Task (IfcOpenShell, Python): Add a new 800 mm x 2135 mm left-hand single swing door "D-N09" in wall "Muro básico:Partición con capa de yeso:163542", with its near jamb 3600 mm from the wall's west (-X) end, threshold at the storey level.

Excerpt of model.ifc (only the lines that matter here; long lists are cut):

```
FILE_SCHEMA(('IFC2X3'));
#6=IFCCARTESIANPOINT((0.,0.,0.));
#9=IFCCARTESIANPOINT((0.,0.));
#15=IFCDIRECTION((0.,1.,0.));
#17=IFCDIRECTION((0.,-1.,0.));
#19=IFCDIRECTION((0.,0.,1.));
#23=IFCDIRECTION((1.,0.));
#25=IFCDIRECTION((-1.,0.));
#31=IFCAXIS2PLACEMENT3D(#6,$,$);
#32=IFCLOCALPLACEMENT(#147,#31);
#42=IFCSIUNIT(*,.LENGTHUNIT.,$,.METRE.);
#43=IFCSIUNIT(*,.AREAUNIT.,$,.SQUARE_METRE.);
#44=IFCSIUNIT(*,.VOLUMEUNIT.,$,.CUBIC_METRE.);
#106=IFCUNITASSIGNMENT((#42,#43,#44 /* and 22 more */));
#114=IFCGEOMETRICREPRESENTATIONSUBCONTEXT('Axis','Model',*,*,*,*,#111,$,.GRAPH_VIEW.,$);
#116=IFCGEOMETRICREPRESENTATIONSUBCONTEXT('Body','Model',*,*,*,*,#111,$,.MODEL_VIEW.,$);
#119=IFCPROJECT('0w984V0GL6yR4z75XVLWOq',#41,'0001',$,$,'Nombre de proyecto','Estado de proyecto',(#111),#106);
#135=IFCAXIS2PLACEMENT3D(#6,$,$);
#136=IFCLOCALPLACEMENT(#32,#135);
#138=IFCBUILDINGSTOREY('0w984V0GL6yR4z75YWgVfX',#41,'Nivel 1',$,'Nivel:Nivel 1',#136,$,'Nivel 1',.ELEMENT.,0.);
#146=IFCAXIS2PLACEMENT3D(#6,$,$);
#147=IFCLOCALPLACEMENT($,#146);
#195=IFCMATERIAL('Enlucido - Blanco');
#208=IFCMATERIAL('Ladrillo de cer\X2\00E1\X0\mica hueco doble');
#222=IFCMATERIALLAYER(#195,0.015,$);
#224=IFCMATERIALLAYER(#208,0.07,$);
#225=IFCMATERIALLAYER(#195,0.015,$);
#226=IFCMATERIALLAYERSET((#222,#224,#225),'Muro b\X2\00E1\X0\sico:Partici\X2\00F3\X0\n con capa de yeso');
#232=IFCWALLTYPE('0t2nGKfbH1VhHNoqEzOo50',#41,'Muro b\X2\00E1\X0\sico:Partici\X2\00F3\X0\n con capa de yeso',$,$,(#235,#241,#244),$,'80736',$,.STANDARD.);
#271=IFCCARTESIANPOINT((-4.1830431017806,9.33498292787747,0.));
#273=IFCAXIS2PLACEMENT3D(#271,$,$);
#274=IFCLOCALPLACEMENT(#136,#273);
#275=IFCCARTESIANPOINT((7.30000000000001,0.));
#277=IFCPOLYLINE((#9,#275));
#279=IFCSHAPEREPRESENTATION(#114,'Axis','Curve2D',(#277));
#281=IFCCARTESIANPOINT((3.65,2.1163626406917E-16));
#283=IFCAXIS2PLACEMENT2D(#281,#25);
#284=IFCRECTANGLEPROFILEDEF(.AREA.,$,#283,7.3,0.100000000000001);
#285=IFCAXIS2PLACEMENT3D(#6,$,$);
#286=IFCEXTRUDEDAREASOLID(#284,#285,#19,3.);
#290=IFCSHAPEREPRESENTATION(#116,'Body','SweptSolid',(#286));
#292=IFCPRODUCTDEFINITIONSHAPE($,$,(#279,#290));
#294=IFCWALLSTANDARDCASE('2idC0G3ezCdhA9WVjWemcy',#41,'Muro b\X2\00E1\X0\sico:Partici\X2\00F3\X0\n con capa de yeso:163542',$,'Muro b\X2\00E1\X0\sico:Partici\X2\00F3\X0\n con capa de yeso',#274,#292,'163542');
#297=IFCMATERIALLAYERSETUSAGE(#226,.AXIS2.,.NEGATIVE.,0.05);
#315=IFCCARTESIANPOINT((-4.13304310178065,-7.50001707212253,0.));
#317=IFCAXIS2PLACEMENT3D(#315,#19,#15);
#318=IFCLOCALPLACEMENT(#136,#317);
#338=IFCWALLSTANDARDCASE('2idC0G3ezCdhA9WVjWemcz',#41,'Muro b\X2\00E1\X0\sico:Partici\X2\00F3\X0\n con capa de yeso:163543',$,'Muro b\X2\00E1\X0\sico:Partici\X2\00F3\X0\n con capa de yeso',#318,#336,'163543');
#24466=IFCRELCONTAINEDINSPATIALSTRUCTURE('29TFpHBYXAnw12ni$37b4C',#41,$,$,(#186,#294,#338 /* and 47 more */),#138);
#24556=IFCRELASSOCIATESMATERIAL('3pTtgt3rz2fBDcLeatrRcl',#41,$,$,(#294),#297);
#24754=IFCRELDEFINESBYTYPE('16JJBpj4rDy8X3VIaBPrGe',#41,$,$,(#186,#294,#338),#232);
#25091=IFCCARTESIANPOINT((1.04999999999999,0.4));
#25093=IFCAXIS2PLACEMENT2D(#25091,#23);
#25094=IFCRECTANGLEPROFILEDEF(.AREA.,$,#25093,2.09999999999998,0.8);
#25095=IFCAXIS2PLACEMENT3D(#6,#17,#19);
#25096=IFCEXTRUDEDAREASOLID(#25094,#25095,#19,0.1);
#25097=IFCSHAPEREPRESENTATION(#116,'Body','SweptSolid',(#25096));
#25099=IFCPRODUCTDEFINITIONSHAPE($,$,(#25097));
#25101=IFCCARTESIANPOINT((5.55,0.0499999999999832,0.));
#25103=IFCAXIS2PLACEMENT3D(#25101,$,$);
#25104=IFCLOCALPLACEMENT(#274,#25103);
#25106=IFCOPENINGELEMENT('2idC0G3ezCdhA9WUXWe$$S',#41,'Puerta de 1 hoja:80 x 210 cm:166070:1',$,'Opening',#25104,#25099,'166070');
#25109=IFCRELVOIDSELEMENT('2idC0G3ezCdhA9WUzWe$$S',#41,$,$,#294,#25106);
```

```python
import numpy as np
import ifcopenshell
import ifcopenshell.api.feature
import ifcopenshell.api.geometry
import ifcopenshell.api.root
import ifcopenshell.api.spatial
import ifcopenshell.api.type
import ifcopenshell.geom
import ifcopenshell.util.element
import ifcopenshell.util.placement
import ifcopenshell.util.representation
import ifcopenshell.util.shape
import ifcopenshell.util.unit

model = ifcopenshell.open("model.ifc")
unit_scale = ifcopenshell.util.unit.calculate_unit_scale(model)
settings = ifcopenshell.geom.settings()


def volume(element):
    """Net volume in cubic metres, openings subtracted."""
    shape = ifcopenshell.geom.create_shape(settings, element)
    return ifcopenshell.util.shape.get_volume(shape.geometry)


wall = model.by_guid("2idC0G3ezCdhA9WVjWemcy")
storey = ifcopenshell.util.element.get_container(wall, ifc_class="IfcBuildingStorey")
context = ifcopenshell.util.representation.get_context(model, "Model", "Body", "MODEL_VIEW")
before = volume(wall)

width, height, from_end, sill = 0.8, 2.135, 3.6, 0.0  # metres

# The wall runs along its own X axis, and the end named is its -X end.
wall_shape = ifcopenshell.geom.create_shape(settings, wall)
x, y, z = ifcopenshell.util.shape.get_vertices(wall_shape.geometry).T
start = x.min() + from_end
face, thickness = float(y.min()), float(y.max() - y.min())
wall_matrix = ifcopenshell.util.placement.get_local_placement(wall.ObjectPlacement)
level = ifcopenshell.util.placement.get_local_placement(storey.ObjectPlacement)[2, 3]


def in_wall(x, y):
    """Placement at x, y metres in the wall's axes, at sill height."""
    matrix = wall_matrix.copy()
    matrix[:, 3] = wall_matrix @ np.array([x / unit_scale, y / unit_scale, 0.0, 1.0])
    matrix[2, 3] = level + sill / unit_scale
    return matrix


# Opening: a box that overshoots both wall faces by 50 mm.
opening = ifcopenshell.api.root.create_entity(model, ifc_class="IfcOpeningElement")
box = ifcopenshell.api.geometry.add_wall_representation(
    model, context=context, length=width, height=height, thickness=thickness + 0.1
)
ifcopenshell.api.geometry.assign_representation(model, product=opening, representation=box)
ifcopenshell.api.geometry.edit_object_placement(model, product=opening, matrix=in_wall(start, face - 0.05), is_si=False)
ifcopenshell.api.feature.add_feature(model, feature=opening, element=wall)

door = ifcopenshell.api.root.create_entity(model, ifc_class="IfcDoor", name="D-N09")
door.OverallWidth, door.OverallHeight = width / unit_scale, height / unit_scale
body = ifcopenshell.api.geometry.add_door_representation(
    model,
    context=context,
    overall_width=door.OverallWidth,
    overall_height=door.OverallHeight,
    operation_type="SINGLE_SWING_LEFT",
    lining_properties={"LiningDepth": thickness / unit_scale, "ThresholdDepth": thickness / unit_scale},
)
ifcopenshell.api.geometry.assign_representation(model, product=door, representation=body)
ifcopenshell.api.spatial.assign_container(model, products=[door], relating_structure=storey)
fills = ifcopenshell.api.feature.add_filling(model, opening=opening, element=door)
fills.OwnerHistory = door.OwnerHistory  # required in IFC2X3

# IFC2X3 keeps the operation on the door style.
style = ifcopenshell.api.root.create_entity(model, ifc_class="IfcDoorStyle", name="D-N09")
style.OperationType, style.ConstructionType = "SINGLE_SWING_LEFT", "NOTDEFINED"
style.ParameterTakesPrecedence = style.Sizeable = False
ifcopenshell.api.type.assign_type(model, related_objects=[door], relating_type=style)

# The lining spans the wall, so the door starts at the wall face.
ifcopenshell.api.geometry.edit_object_placement(model, product=door, matrix=in_wall(start, face), is_si=False)

after = volume(wall)

print(f"wall volume {before:.3f} -> {after:.3f} m3")

model.write("model-out.ifc")
```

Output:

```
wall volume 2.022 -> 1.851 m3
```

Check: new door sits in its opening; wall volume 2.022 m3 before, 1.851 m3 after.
